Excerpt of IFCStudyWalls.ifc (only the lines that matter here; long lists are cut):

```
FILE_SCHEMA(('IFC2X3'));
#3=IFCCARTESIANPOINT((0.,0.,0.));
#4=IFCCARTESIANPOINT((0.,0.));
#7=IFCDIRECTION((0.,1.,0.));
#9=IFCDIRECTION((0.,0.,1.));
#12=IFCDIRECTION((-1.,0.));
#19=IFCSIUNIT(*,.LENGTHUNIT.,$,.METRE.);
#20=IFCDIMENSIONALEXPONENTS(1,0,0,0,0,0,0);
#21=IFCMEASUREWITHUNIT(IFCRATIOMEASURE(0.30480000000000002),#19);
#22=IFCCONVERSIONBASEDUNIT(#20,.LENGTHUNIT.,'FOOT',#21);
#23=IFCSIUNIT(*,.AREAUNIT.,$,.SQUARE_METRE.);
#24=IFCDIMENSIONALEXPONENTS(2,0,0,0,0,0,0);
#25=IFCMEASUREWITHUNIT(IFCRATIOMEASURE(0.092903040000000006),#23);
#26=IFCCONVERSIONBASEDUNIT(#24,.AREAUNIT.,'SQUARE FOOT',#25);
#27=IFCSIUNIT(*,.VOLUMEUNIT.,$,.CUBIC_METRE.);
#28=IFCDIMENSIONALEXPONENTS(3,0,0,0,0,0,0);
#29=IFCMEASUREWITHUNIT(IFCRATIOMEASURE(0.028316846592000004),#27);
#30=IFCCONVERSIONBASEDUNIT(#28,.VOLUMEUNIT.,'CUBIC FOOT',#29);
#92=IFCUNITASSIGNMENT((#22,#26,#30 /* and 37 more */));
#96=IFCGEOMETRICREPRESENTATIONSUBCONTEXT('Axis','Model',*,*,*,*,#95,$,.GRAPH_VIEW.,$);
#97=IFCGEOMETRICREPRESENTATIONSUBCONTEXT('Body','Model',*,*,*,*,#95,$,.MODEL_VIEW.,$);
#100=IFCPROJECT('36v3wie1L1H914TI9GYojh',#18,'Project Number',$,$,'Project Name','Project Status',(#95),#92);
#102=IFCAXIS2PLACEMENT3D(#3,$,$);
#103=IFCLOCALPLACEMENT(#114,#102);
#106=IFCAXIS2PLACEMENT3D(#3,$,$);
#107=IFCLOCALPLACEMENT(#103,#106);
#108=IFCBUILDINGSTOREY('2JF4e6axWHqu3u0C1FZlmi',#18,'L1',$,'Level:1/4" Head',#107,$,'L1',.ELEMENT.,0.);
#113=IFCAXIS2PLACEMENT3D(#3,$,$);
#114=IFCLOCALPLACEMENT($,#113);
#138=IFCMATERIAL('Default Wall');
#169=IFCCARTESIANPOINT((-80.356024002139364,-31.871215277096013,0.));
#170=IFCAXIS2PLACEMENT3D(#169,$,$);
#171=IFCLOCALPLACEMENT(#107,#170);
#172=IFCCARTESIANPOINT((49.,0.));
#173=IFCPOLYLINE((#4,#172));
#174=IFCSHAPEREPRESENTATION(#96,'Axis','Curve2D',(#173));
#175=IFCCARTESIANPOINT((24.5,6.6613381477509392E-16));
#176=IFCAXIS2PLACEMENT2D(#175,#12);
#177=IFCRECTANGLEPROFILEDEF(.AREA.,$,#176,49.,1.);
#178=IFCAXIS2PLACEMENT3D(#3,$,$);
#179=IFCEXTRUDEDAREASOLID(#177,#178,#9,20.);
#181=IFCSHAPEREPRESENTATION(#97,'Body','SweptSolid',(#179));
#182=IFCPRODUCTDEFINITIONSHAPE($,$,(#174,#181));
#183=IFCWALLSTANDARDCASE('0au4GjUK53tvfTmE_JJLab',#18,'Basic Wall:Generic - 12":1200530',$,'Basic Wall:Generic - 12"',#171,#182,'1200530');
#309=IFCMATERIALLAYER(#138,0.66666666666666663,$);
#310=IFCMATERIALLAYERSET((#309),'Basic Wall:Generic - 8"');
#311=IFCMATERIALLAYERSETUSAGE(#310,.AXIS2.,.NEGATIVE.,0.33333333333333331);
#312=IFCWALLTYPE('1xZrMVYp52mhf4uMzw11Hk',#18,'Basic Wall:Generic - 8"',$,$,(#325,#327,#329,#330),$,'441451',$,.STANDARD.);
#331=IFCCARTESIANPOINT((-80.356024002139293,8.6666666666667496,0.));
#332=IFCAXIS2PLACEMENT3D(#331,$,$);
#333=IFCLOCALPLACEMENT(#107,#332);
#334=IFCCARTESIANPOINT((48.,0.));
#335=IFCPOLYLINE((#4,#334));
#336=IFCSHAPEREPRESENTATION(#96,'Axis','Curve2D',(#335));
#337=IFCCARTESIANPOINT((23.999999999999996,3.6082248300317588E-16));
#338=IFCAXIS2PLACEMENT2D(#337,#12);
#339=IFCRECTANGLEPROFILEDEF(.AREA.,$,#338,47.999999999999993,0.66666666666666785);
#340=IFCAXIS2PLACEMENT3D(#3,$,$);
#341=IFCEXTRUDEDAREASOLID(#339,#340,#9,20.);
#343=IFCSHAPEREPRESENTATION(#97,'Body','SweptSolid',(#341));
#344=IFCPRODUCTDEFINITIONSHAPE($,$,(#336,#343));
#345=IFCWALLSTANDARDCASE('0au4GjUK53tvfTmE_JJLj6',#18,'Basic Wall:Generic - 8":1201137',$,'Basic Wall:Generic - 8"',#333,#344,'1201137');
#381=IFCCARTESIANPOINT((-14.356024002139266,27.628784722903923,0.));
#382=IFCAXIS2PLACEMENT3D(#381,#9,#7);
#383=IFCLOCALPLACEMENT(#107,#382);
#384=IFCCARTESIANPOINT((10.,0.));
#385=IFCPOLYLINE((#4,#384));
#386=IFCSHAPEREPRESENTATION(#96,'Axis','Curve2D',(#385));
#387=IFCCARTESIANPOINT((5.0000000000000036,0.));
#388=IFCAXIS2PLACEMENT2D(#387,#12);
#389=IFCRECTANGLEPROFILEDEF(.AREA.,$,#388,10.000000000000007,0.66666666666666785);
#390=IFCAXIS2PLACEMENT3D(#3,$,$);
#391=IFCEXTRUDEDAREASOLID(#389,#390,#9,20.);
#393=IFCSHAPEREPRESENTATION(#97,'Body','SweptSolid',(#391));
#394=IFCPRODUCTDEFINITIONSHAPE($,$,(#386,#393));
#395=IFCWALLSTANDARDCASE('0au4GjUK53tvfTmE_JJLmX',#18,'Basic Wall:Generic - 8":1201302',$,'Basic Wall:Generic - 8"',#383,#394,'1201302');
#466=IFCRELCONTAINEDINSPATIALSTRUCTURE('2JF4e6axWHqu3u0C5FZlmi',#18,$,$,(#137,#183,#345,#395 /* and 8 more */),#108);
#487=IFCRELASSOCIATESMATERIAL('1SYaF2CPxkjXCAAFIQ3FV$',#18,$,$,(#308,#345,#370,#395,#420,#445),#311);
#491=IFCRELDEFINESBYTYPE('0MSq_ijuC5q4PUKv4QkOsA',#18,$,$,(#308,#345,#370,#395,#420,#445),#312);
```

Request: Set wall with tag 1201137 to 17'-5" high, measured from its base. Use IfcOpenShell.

```python
import ifcopenshell
import ifcopenshell.geom
import ifcopenshell.util.representation
import ifcopenshell.util.shape
import ifcopenshell.util.unit

model = ifcopenshell.open("IFCStudyWalls.ifc")
unit_scale = ifcopenshell.util.unit.calculate_unit_scale(model)
settings = ifcopenshell.geom.settings()


def volume(element):
    """Net volume in cubic metres, openings subtracted."""
    shape = ifcopenshell.geom.create_shape(settings, element)
    return ifcopenshell.util.shape.get_volume(shape.geometry)


wall = model.by_guid("0au4GjUK53tvfTmE_JJLj6")
before = volume(wall)

body = ifcopenshell.util.representation.get_representation(wall, "Model", "Body")
solid = body.Items[0]
old_height = solid.Depth
solid.Depth = 209 * 0.0254 / unit_scale
after = volume(wall)

print(f"height {old_height:g} -> {solid.Depth:g}, volume {before:.3f} -> {after:.3f} m3")

model.write("IFCStudyWalls-out.ifc")
```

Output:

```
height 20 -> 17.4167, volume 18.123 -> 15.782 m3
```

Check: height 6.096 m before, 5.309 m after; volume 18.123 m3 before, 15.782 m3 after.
